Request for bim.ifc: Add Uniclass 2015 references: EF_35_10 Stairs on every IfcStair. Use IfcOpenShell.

First a look at what the model holds.

```python
import ifcopenshell

model = ifcopenshell.open("bim.ifc")
print(model.schema)
print("classifications:", [c.Name for c in model.by_type("IfcClassification")])
for ifc_class in ("IfcDoor", "IfcRoof", "IfcStair", "IfcWall", "IfcWindow"):
    print(ifc_class, len(model.by_type(ifc_class)))
```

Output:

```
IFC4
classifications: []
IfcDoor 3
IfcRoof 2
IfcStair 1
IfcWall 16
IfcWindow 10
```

```python
import ifcopenshell
import ifcopenshell.api.classification

model = ifcopenshell.open("bim.ifc")

system = ifcopenshell.api.classification.add_classification(model, classification="Uniclass 2015")

codes = {
    "IfcStair": ("EF_35_10", "Stairs"),
}
for ifc_class, (code, name) in codes.items():
    products = model.by_type(ifc_class)
    ifcopenshell.api.classification.add_reference(
        model, products=products, classification=system, identification=code, name=name
    )
    print(code, len(products))

model.write("bim_updated.ifc")
```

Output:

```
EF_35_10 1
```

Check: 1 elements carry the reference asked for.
